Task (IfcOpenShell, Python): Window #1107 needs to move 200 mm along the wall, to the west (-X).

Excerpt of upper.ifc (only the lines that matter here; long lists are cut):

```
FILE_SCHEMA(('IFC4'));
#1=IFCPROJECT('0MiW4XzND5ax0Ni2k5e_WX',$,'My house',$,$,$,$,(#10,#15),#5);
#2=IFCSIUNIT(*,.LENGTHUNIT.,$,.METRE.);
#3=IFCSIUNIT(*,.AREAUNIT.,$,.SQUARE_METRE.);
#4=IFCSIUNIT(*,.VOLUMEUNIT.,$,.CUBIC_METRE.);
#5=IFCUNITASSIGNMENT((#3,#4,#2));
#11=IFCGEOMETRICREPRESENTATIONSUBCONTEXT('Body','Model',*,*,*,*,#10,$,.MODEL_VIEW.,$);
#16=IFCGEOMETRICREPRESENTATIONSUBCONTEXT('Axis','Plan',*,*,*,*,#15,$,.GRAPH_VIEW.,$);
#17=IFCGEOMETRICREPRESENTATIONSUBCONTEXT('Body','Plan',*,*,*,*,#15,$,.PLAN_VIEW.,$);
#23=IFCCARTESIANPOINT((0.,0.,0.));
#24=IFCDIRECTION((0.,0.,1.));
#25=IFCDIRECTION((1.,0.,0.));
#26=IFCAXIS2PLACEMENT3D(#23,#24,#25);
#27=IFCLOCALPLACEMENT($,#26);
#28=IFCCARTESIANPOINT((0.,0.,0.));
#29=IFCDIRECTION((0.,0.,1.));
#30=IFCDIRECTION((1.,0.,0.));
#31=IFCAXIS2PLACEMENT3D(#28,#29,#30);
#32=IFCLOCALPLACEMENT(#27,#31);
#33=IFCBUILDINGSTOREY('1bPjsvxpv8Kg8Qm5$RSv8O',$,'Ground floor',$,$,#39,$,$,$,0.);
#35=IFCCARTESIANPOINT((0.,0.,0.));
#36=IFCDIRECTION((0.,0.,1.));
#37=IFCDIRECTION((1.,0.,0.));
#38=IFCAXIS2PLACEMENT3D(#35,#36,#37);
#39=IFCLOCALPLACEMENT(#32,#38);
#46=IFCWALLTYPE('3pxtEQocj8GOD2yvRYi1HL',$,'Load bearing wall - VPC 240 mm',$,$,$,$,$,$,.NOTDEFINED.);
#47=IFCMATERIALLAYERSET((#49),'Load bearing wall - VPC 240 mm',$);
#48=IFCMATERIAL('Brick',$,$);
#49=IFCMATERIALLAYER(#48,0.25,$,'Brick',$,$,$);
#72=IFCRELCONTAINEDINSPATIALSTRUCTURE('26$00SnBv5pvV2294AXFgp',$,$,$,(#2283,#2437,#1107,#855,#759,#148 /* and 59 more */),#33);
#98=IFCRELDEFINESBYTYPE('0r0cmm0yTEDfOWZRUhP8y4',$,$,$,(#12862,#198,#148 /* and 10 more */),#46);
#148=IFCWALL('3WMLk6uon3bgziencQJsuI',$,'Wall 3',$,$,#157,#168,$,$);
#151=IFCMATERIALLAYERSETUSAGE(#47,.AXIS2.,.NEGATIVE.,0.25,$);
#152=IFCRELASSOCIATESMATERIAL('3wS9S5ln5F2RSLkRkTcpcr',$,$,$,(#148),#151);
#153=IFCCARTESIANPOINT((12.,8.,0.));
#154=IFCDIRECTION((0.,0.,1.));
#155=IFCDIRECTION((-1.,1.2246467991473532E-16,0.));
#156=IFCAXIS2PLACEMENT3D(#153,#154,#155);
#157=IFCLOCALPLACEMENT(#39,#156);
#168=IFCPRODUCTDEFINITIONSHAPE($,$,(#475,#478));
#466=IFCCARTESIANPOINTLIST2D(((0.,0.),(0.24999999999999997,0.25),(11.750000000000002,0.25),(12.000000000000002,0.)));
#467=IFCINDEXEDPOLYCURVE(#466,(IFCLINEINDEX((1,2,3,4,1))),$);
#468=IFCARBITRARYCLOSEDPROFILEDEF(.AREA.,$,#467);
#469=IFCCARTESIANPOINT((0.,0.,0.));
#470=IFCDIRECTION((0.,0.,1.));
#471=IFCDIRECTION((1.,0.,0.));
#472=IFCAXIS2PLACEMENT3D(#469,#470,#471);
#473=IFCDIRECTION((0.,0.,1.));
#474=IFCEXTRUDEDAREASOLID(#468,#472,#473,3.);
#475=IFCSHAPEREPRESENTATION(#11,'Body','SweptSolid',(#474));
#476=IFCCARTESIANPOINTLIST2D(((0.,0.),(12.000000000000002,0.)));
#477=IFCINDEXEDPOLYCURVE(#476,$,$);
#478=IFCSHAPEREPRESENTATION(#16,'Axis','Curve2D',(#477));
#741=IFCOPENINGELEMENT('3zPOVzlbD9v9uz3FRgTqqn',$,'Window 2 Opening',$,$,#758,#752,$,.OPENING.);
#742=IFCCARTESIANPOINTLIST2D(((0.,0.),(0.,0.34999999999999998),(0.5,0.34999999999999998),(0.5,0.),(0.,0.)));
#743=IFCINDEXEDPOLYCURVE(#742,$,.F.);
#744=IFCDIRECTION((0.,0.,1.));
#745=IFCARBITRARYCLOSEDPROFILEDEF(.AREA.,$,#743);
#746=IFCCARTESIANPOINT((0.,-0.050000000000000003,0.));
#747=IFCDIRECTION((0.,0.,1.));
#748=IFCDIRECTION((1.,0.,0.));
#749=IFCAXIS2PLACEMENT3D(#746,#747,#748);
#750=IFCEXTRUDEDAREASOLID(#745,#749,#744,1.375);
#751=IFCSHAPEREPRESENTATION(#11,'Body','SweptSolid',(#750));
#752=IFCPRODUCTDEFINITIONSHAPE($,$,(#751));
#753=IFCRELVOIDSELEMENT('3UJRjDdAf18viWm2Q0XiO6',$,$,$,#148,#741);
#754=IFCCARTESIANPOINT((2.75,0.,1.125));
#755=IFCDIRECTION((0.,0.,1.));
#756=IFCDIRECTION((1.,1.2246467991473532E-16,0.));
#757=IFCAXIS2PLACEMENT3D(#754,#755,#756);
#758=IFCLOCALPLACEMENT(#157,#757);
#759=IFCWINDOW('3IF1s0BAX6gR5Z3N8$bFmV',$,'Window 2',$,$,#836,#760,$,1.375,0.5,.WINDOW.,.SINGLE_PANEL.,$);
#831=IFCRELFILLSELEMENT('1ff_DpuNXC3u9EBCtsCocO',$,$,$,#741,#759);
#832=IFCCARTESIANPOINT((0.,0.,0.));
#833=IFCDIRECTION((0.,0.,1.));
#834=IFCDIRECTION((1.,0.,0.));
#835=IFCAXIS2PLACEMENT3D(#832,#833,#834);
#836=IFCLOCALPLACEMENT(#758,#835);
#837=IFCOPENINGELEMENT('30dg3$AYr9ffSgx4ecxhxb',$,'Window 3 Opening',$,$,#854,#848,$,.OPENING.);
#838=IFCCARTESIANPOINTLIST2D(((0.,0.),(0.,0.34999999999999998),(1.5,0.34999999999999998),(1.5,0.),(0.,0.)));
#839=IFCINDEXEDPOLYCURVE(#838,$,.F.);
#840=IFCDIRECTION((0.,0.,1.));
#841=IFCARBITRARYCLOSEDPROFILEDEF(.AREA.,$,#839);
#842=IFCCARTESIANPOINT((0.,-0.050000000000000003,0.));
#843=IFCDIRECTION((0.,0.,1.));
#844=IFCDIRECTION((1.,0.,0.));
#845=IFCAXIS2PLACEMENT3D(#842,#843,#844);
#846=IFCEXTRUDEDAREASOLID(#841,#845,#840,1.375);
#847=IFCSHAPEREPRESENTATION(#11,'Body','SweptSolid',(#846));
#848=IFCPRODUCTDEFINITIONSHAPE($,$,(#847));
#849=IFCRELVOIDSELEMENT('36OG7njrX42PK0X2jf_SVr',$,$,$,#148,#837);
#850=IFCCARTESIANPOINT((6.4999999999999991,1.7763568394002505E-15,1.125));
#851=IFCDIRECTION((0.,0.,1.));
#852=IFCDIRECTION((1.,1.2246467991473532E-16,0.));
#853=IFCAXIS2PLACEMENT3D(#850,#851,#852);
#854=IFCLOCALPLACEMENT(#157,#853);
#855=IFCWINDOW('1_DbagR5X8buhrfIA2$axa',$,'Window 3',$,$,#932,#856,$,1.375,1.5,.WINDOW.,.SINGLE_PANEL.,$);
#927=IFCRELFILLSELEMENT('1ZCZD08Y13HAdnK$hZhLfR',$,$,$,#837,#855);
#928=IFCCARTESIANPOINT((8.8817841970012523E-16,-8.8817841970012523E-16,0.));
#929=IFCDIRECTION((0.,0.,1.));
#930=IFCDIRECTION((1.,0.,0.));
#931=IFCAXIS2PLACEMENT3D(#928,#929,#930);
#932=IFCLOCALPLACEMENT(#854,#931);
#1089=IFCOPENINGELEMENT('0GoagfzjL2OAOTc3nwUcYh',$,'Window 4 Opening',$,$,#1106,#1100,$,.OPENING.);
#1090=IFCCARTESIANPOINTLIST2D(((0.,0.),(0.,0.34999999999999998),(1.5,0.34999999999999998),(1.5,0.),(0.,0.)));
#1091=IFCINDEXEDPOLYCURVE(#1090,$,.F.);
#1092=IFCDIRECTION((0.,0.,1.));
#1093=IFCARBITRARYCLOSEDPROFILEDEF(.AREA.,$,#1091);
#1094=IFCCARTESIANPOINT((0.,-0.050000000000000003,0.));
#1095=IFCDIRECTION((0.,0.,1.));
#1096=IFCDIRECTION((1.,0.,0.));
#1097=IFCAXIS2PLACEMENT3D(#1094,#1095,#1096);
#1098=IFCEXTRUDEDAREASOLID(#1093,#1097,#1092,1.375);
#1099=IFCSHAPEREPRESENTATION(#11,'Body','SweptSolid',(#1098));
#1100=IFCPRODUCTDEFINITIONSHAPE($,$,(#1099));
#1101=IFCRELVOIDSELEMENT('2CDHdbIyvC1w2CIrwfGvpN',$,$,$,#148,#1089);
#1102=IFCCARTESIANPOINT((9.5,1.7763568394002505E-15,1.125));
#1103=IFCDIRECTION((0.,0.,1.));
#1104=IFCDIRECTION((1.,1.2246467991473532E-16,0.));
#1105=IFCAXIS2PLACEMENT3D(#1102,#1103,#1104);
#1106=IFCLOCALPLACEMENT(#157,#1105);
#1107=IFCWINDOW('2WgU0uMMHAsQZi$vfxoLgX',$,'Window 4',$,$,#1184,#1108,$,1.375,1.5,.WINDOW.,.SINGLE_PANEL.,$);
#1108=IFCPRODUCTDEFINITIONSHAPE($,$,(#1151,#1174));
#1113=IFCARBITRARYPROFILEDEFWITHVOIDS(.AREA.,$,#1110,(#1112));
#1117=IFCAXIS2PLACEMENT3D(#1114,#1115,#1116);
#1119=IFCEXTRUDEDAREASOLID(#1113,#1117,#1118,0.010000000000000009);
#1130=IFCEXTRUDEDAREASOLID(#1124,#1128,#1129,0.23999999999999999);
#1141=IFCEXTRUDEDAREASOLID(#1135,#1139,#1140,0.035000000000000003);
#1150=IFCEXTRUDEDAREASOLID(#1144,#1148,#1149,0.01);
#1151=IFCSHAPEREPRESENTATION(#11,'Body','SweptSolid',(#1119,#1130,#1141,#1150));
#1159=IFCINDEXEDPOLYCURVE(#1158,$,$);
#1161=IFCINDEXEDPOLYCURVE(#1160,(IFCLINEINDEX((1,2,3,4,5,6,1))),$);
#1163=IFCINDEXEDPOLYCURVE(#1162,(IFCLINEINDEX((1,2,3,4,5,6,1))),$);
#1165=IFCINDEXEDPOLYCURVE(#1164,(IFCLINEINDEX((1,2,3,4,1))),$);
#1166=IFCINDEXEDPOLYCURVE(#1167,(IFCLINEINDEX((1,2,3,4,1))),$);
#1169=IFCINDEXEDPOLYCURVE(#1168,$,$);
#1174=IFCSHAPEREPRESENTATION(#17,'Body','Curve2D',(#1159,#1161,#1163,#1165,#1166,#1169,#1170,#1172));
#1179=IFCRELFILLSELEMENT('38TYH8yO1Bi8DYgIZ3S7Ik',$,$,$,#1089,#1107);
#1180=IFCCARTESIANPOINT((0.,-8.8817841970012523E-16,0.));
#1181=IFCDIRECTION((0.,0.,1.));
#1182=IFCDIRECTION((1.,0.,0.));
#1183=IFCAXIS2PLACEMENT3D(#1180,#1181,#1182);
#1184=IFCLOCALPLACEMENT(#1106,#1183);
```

```python
import ifcopenshell
import ifcopenshell.api.geometry
import ifcopenshell.util.placement
import ifcopenshell.util.unit

model = ifcopenshell.open("upper.ifc")
unit_scale = ifcopenshell.util.unit.calculate_unit_scale(model)

window = model.by_guid("2WgU0uMMHAsQZi$vfxoLgX")
opening = window.FillsVoids[0].RelatingOpeningElement
wall = opening.VoidsElements[0].RelatingBuildingElement

wall_matrix = ifcopenshell.util.placement.get_local_placement(wall.ObjectPlacement)
shift = wall_matrix[:3, 0] * 0.2 / unit_scale
before = ifcopenshell.util.placement.get_local_placement(window.ObjectPlacement)[:3, 3].copy()

# The window is placed relative to its opening, so it follows when the opening moves.
matrix = ifcopenshell.util.placement.get_local_placement(opening.ObjectPlacement)
matrix[:3, 3] += shift
ifcopenshell.api.geometry.edit_object_placement(
    model, product=opening, matrix=matrix, is_si=False, should_transform_children=True
)

after = ifcopenshell.util.placement.get_local_placement(window.ObjectPlacement)[:3, 3]
print("window moved by", (after - before).round(3) + 0.0)

model.write("upper_v2.ifc")
```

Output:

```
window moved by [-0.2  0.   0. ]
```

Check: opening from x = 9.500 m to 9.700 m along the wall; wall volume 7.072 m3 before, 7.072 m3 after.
